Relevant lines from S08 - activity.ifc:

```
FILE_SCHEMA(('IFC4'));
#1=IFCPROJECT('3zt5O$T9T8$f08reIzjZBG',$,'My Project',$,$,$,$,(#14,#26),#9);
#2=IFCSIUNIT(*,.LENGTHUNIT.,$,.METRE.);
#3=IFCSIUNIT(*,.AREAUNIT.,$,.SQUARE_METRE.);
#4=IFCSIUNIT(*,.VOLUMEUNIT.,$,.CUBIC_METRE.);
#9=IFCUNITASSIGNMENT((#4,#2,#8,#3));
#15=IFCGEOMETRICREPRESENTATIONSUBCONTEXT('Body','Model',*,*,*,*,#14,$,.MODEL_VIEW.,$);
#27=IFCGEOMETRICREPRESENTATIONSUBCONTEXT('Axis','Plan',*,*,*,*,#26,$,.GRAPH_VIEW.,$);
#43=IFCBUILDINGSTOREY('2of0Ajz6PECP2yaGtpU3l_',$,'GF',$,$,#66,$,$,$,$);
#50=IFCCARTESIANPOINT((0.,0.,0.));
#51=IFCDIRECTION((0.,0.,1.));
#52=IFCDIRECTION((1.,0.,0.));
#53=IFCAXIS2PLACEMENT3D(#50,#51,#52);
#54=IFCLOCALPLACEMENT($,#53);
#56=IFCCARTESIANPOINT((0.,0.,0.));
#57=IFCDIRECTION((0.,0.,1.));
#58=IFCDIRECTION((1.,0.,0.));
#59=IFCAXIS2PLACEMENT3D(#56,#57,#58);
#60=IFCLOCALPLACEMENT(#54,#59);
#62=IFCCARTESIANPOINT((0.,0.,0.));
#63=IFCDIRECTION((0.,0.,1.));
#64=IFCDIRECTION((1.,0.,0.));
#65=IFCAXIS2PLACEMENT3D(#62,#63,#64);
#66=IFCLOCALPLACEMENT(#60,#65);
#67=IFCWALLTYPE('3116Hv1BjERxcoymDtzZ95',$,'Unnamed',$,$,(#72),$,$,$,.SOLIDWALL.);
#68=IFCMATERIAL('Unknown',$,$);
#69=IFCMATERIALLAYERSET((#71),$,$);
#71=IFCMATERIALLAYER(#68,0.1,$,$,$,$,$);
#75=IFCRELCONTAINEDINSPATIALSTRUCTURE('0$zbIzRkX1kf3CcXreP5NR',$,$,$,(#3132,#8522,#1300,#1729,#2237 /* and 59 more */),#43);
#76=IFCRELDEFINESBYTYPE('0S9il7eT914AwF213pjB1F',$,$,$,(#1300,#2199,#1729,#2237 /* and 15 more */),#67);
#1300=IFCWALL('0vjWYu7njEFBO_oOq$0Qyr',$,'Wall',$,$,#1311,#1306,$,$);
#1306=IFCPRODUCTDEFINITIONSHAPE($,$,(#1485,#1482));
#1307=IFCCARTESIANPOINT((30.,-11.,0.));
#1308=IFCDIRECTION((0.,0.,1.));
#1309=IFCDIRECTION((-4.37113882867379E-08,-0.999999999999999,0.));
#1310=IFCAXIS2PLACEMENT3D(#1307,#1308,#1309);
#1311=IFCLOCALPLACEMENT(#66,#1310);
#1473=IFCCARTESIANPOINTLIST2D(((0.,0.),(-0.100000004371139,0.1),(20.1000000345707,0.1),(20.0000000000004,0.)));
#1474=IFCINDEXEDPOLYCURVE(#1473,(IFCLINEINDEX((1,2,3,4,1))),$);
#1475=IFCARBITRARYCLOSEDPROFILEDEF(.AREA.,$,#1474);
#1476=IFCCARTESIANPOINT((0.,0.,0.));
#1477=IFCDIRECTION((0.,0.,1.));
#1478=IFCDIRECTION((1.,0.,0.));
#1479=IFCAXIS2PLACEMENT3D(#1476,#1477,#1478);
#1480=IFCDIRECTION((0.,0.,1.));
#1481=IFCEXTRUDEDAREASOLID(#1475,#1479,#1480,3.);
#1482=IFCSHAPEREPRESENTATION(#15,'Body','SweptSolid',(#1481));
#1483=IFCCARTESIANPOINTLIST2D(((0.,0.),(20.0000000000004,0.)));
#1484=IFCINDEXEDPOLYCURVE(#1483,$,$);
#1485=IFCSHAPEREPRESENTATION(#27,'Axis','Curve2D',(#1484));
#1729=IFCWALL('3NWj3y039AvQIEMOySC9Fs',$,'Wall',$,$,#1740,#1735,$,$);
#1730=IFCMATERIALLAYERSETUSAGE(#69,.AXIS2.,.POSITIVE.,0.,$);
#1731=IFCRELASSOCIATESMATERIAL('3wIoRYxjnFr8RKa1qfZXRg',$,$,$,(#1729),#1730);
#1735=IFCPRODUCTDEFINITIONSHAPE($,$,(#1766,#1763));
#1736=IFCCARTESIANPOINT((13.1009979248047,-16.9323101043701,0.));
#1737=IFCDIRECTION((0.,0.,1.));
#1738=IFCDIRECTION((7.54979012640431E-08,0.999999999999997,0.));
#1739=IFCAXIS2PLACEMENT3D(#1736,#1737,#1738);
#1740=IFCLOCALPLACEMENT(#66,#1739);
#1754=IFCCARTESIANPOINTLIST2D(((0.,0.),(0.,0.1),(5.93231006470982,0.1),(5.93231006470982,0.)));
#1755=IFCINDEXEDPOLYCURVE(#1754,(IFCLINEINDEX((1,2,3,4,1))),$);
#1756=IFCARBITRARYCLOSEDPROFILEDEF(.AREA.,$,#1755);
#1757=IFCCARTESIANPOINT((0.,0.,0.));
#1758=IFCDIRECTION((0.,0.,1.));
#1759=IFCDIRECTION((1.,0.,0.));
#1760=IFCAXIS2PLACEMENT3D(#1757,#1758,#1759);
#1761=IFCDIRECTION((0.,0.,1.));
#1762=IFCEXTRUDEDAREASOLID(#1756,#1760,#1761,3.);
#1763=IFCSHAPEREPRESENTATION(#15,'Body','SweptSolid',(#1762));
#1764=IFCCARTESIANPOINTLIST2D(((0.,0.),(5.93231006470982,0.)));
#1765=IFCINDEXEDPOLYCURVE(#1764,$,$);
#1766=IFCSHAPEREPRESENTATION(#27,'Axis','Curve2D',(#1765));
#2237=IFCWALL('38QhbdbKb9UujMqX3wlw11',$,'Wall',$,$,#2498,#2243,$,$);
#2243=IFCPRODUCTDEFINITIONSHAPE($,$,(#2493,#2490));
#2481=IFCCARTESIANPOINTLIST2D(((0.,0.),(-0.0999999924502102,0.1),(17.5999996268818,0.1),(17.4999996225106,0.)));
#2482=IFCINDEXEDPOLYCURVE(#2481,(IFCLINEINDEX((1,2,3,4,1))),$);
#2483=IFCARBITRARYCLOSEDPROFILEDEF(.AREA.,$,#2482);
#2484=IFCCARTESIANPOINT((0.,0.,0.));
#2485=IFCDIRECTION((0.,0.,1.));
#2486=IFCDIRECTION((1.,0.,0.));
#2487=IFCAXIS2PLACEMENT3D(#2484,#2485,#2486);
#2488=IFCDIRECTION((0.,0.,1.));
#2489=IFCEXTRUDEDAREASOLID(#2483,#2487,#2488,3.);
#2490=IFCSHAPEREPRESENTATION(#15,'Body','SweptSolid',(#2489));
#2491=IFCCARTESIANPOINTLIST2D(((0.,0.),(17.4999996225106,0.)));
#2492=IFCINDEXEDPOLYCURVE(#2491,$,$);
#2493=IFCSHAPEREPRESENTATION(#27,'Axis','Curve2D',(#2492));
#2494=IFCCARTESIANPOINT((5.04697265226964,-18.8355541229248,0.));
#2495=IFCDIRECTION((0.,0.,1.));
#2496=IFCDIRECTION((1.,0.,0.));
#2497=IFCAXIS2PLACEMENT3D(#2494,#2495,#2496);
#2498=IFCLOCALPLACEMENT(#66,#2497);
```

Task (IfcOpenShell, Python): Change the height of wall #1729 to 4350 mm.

```python
import ifcopenshell
import ifcopenshell.geom
import ifcopenshell.util.representation
import ifcopenshell.util.shape
import ifcopenshell.util.unit

model = ifcopenshell.open("S08 - activity.ifc")
unit_scale = ifcopenshell.util.unit.calculate_unit_scale(model)
settings = ifcopenshell.geom.settings()


def volume(element):
    """Net volume in cubic metres, openings subtracted."""
    shape = ifcopenshell.geom.create_shape(settings, element)
    return ifcopenshell.util.shape.get_volume(shape.geometry)


wall = model.by_guid("3NWj3y039AvQIEMOySC9Fs")
before = volume(wall)

body = ifcopenshell.util.representation.get_representation(wall, "Model", "Body")
solid = body.Items[0]
old_height = solid.Depth
solid.Depth = 4.35 / unit_scale
after = volume(wall)

print(f"height {old_height:g} -> {solid.Depth:g}, volume {before:.3f} -> {after:.3f} m3")

model.write("S08 - activity-out.ifc")
```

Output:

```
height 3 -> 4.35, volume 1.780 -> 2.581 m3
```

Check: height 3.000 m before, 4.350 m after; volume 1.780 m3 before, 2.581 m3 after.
